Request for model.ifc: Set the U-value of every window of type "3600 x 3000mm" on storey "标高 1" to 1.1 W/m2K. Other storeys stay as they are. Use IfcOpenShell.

First a look at what the model holds.

```python
import ifcopenshell
import ifcopenshell.util.element

model = ifcopenshell.open("model.ifc")
print(model.schema)
storey = next(s for s in model.by_type("IfcBuildingStorey") if s.Name == "标高 1")
windows = [e for e in ifcopenshell.util.element.get_decomposition(storey) if e.is_a("IfcWindow")]
seen = {}
for e in windows:
    element_type = ifcopenshell.util.element.get_type(e)
    key = (element_type.Name if element_type != e and element_type else None, ifcopenshell.util.element.get_pset(e, "Pset_WindowCommon", "ThermalTransmittance"))
    seen[key] = seen.get(key, 0) + 1
for (name, value), count in sorted(seen.items(), key=str):
    print(count, "x", name, "|", value)
```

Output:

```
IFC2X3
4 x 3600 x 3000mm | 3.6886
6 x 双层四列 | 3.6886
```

```python
import ifcopenshell
import ifcopenshell.api.pset
import ifcopenshell.util.element

model = ifcopenshell.open("model.ifc")

storey = next(s for s in model.by_type("IfcBuildingStorey") if s.Name == "标高 1")
windows = [e for e in ifcopenshell.util.element.get_decomposition(storey) if e.is_a("IfcWindow")]

count = 0
for e in windows:
    element_type = ifcopenshell.util.element.get_type(e)
    if element_type in (None, e) or element_type.Name != "3600 x 3000mm":
        continue
    # add_pset returns the element's existing set when there is one.
    pset = ifcopenshell.api.pset.add_pset(model, product=e, name="Pset_WindowCommon")
    ifcopenshell.api.pset.edit_pset(model, pset=pset, properties={"ThermalTransmittance": 1.1})
    count += 1

print(count, "windows updated")

model.write("model_v2.ifc")
```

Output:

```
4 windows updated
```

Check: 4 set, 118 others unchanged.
